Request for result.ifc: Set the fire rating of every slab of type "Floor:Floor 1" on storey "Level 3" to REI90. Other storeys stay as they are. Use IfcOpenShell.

First a look at what the model holds.

```python
import ifcopenshell
import ifcopenshell.util.element

model = ifcopenshell.open("result.ifc")
print(model.schema)
storey = next(s for s in model.by_type("IfcBuildingStorey") if s.Name == "Level 3")
slabs = [e for e in ifcopenshell.util.element.get_decomposition(storey) if e.is_a("IfcSlab")]
seen = {}
for e in slabs:
    element_type = ifcopenshell.util.element.get_type(e)
    key = (element_type.Name if element_type != e and element_type else None, ifcopenshell.util.element.get_pset(e, "Pset_SlabCommon", "FireRating"))
    seen[key] = seen.get(key, 0) + 1
for (name, value), count in sorted(seen.items(), key=str):
    print(count, "x", name, "|", value)
```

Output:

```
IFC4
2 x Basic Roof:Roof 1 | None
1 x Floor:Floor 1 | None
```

```python
import ifcopenshell
import ifcopenshell.api.pset
import ifcopenshell.util.element

model = ifcopenshell.open("result.ifc")

storey = next(s for s in model.by_type("IfcBuildingStorey") if s.Name == "Level 3")
slabs = [e for e in ifcopenshell.util.element.get_decomposition(storey) if e.is_a("IfcSlab")]

count = 0
for e in slabs:
    element_type = ifcopenshell.util.element.get_type(e)
    if element_type in (None, e) or element_type.Name != "Floor:Floor 1":
        continue
    # add_pset returns the element's existing set when there is one.
    pset = ifcopenshell.api.pset.add_pset(model, product=e, name="Pset_SlabCommon")
    ifcopenshell.api.pset.edit_pset(model, pset=pset, properties={"FireRating": "REI90"})
    count += 1

print(count, "slabs updated")

model.write("result-out.ifc")
```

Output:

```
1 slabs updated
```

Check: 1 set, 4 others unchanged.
